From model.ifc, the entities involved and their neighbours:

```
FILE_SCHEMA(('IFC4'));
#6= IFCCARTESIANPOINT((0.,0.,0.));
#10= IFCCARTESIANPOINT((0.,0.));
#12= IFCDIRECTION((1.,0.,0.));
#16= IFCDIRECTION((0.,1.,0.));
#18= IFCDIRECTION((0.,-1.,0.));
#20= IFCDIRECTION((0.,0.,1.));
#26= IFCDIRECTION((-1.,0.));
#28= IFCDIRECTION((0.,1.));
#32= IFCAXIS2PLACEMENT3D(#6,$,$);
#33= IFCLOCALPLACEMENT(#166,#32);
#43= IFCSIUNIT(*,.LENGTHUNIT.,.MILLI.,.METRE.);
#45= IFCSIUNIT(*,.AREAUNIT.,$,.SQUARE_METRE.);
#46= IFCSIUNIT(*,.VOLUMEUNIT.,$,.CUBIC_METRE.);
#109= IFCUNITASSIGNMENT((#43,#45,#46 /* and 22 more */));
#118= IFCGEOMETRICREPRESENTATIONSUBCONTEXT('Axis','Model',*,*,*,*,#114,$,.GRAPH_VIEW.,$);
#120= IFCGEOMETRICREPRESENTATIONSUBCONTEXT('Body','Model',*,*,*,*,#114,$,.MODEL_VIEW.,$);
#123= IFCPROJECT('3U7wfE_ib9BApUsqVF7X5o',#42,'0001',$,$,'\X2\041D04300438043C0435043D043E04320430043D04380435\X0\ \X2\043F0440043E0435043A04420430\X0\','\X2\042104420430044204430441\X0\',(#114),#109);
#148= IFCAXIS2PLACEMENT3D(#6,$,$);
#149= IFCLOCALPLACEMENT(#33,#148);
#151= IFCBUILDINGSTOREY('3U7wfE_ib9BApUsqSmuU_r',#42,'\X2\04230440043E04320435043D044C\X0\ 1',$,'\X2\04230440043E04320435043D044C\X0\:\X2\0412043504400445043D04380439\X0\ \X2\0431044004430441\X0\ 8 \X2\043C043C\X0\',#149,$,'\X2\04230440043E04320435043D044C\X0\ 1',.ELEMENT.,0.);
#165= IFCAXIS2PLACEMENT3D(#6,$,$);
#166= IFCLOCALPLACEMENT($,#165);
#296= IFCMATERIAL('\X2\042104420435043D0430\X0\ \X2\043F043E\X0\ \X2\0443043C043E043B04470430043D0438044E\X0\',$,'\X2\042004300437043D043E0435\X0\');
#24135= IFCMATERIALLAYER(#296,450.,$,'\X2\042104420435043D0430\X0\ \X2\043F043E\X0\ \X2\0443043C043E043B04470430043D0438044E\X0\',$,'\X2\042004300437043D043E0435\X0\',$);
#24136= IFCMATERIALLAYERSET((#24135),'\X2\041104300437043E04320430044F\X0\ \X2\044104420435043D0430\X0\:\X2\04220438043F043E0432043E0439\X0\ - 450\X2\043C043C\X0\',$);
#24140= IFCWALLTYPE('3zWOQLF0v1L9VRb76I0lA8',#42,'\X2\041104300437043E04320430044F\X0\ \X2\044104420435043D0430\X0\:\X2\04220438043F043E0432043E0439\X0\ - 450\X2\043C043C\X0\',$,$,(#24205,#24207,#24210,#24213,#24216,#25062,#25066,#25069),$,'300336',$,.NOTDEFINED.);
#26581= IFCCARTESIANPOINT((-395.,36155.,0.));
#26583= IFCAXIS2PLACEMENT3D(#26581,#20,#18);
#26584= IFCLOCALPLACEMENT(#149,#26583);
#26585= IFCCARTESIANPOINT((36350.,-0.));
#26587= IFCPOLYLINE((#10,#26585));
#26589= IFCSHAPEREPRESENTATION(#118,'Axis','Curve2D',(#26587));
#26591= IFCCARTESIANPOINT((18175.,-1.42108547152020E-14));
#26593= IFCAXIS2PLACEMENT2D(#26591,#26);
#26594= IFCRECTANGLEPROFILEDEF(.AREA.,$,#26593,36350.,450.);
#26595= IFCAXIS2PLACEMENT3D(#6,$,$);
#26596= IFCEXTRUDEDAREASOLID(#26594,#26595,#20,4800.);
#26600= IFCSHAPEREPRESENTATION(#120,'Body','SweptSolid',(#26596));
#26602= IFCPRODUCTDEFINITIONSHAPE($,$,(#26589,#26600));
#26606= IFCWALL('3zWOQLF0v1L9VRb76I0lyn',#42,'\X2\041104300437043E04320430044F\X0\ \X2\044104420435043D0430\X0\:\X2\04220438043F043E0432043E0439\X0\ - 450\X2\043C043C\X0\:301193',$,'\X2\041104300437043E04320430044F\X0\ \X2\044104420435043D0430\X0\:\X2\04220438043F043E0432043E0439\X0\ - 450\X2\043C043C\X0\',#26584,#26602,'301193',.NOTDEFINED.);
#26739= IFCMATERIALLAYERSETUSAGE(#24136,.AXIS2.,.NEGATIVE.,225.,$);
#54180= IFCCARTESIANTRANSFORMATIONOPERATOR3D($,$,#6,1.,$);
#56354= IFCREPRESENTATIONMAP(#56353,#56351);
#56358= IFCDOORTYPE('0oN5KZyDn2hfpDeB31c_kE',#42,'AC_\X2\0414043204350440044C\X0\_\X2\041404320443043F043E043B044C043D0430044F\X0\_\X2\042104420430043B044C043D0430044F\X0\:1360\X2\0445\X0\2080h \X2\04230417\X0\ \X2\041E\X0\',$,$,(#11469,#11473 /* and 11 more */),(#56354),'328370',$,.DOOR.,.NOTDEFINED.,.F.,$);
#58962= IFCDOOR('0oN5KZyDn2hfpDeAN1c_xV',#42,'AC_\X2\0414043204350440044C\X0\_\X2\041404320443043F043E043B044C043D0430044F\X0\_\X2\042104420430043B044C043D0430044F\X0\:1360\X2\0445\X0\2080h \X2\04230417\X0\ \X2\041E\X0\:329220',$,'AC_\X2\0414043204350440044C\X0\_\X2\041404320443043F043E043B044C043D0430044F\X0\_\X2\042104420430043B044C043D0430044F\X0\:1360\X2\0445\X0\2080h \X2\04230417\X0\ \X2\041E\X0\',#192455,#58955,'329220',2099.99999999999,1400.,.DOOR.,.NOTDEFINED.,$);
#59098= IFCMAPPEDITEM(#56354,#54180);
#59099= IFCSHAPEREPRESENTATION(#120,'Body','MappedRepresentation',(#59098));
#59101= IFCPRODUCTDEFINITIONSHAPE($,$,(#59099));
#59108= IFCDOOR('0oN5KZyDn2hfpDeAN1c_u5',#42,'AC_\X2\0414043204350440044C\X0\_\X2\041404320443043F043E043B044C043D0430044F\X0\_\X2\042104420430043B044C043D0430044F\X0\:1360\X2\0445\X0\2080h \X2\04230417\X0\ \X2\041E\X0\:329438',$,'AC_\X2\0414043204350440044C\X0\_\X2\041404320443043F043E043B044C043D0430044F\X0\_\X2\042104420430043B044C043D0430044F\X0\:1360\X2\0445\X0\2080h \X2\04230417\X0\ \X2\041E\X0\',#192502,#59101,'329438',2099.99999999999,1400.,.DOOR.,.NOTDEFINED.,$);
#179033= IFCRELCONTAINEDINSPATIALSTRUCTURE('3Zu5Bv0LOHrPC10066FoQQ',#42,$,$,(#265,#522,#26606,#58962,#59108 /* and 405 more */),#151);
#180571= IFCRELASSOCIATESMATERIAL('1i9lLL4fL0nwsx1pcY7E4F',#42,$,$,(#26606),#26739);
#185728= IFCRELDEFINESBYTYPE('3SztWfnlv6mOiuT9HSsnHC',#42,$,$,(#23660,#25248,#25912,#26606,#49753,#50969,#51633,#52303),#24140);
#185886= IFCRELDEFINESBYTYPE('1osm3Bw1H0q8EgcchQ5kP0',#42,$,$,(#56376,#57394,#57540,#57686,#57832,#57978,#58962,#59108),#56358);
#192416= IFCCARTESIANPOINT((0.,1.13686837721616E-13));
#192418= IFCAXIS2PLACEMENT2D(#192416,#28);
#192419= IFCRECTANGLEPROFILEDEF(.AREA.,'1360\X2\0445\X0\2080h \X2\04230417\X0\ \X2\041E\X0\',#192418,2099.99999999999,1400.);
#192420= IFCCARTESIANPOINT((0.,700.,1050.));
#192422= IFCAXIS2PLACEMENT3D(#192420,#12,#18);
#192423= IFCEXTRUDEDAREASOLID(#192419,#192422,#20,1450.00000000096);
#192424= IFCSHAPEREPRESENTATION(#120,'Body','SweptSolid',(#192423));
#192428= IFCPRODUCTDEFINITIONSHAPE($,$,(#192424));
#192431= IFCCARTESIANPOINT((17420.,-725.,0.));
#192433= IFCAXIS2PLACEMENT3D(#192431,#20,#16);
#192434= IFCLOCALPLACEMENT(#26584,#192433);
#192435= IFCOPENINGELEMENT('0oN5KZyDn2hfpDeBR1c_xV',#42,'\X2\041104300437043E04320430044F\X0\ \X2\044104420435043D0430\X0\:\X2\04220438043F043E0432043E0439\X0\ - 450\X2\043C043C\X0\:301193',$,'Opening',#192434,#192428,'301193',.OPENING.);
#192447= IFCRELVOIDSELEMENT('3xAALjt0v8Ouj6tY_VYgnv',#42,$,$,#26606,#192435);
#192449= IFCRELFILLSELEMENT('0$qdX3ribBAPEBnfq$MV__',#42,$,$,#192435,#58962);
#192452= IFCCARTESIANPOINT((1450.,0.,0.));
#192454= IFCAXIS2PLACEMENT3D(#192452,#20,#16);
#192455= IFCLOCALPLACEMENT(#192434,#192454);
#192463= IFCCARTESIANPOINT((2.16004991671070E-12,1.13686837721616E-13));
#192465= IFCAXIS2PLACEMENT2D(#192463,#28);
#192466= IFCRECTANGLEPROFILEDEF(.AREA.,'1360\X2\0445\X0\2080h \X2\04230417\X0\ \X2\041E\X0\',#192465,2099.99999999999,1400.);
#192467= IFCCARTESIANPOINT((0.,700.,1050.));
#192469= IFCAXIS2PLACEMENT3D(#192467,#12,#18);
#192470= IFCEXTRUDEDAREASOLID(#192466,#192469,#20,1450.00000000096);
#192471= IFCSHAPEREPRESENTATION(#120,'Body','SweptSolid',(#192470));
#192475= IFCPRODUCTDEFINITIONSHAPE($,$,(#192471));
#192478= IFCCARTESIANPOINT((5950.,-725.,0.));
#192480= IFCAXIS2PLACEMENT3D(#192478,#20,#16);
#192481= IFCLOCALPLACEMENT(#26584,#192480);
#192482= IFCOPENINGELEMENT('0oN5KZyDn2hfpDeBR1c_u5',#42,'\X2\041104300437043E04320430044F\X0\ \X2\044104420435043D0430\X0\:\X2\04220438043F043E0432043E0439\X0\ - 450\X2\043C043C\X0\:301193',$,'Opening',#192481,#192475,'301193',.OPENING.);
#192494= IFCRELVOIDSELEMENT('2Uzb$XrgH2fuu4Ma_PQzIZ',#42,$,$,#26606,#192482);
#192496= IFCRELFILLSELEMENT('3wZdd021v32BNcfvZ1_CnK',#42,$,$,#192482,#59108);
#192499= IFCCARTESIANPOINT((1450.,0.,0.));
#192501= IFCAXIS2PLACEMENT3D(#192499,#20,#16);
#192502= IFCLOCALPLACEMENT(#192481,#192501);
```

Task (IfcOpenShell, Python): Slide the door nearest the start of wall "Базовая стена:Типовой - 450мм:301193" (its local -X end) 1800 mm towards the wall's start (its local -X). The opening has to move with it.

```python
import ifcopenshell
import ifcopenshell.api.geometry
import ifcopenshell.util.placement
import ifcopenshell.util.unit

model = ifcopenshell.open("model.ifc")
unit_scale = ifcopenshell.util.unit.calculate_unit_scale(model)

door = model.by_guid("0oN5KZyDn2hfpDeAN1c_u5")
opening = door.FillsVoids[0].RelatingOpeningElement
wall = opening.VoidsElements[0].RelatingBuildingElement

wall_matrix = ifcopenshell.util.placement.get_local_placement(wall.ObjectPlacement)
shift = wall_matrix[:3, 0] * -1.8 / unit_scale
before = ifcopenshell.util.placement.get_local_placement(door.ObjectPlacement)[:3, 3].copy()

# The door is placed relative to its opening, so it follows when the opening moves.
matrix = ifcopenshell.util.placement.get_local_placement(opening.ObjectPlacement)
matrix[:3, 3] += shift
ifcopenshell.api.geometry.edit_object_placement(
    model, product=opening, matrix=matrix, is_si=False, should_transform_children=True
)

after = ifcopenshell.util.placement.get_local_placement(door.ObjectPlacement)[:3, 3]
print("door moved by", (after - before).round(3) + 0.0)

model.write("model_rev.ifc")
```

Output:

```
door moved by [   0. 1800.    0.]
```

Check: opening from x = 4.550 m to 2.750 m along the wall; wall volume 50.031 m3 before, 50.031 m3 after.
